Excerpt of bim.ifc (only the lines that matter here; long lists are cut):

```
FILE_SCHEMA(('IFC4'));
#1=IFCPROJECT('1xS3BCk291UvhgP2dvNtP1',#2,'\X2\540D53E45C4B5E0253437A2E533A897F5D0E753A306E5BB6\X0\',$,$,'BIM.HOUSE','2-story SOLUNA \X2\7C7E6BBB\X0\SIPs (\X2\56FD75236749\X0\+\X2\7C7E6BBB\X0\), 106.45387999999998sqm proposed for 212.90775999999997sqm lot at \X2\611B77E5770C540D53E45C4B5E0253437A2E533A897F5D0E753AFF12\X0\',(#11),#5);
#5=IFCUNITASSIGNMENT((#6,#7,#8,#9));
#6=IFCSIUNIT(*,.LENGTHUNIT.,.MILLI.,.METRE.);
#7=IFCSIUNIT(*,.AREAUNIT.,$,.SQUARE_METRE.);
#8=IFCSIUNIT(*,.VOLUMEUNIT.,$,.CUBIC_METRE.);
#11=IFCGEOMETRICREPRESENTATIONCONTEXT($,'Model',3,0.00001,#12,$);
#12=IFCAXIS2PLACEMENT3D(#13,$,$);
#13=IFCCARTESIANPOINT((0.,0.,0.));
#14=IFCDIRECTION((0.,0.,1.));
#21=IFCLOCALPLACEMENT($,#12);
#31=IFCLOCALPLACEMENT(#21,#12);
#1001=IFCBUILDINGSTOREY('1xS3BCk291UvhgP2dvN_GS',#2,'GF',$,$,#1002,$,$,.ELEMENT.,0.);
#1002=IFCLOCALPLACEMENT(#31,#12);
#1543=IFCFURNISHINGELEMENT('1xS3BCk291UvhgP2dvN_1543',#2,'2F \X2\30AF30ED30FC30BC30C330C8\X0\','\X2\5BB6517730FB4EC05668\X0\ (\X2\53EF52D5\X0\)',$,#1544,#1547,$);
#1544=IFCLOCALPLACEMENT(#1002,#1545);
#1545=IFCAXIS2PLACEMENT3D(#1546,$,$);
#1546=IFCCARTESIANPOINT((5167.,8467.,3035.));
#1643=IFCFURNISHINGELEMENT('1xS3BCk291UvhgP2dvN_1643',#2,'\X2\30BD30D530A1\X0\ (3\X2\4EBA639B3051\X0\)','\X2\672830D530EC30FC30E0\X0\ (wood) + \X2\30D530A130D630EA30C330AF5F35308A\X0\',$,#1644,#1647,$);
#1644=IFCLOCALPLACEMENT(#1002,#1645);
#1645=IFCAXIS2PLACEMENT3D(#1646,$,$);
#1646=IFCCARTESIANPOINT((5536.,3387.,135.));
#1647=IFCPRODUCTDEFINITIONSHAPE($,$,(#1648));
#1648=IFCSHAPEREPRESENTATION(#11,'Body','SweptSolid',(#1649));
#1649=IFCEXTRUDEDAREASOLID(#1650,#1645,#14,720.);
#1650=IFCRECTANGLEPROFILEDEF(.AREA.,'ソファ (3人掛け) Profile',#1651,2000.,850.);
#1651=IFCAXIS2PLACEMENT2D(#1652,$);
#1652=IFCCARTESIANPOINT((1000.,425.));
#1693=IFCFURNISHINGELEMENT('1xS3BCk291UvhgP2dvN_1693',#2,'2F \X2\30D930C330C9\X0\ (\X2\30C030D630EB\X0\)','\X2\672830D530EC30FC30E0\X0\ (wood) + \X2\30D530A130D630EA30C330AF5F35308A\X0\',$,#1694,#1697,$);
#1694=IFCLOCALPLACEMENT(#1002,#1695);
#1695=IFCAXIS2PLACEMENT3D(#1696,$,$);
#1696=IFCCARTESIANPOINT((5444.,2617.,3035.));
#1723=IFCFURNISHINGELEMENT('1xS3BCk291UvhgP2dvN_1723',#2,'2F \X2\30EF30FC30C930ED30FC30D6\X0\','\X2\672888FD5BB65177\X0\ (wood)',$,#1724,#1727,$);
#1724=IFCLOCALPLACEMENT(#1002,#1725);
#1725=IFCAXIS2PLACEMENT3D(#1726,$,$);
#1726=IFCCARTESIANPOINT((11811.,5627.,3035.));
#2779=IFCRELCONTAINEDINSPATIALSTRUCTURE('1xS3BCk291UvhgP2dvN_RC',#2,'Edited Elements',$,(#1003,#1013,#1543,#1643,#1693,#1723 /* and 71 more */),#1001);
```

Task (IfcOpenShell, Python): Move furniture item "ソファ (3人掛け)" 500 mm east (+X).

```python
import ifcopenshell
import ifcopenshell.api.geometry
import ifcopenshell.util.placement
import ifcopenshell.util.unit

model = ifcopenshell.open("bim.ifc")
unit_scale = ifcopenshell.util.unit.calculate_unit_scale(model)

item = model.by_guid("1xS3BCk291UvhgP2dvN_1643")
matrix = ifcopenshell.util.placement.get_local_placement(item.ObjectPlacement)
matrix[0, 3] += 0.5 / unit_scale
ifcopenshell.api.geometry.edit_object_placement(model, product=item, matrix=matrix, is_si=False)

print(ifcopenshell.util.placement.get_local_placement(item.ObjectPlacement).round(3) + 0.0)

model.write("bim_rev.ifc")
```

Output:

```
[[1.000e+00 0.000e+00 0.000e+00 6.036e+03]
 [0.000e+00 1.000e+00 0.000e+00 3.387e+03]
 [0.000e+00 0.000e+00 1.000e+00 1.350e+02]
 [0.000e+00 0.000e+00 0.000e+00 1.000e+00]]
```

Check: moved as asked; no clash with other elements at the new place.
